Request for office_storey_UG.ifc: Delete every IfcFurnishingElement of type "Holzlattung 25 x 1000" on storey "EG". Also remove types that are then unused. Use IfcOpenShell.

First a look at what the model holds.

```python
import ifcopenshell
import ifcopenshell.util.element

model = ifcopenshell.open("office_storey_UG.ifc")
print(model.schema)
storey = next(s for s in model.by_type("IfcBuildingStorey") if s.Name == "EG")
furniture = [e for e in ifcopenshell.util.element.get_decomposition(storey) if e.is_a("IfcFurnishingElement")]
seen = {}
for e in furniture:
    element_type = ifcopenshell.util.element.get_type(e)
    name = element_type.Name if element_type not in (None, e) else None
    seen[name] = seen.get(name, 0) + 1
for name, count in sorted(seen.items(), key=str):
    print(count, "x", name)
```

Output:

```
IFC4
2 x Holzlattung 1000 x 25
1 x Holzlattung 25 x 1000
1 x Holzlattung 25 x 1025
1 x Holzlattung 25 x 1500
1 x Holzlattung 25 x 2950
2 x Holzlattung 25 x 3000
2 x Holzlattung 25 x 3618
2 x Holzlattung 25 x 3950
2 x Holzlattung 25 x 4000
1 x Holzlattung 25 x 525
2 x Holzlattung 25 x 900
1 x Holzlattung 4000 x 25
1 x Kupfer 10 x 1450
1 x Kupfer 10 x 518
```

```python
import ifcopenshell
import ifcopenshell.api.root
import ifcopenshell.util.element

model = ifcopenshell.open("office_storey_UG.ifc")

storey = next(s for s in model.by_type("IfcBuildingStorey") if s.Name == "EG")
furniture = [e for e in ifcopenshell.util.element.get_decomposition(storey) if e.is_a("IfcFurnishingElement")]
targets = [e for e in furniture if (t := ifcopenshell.util.element.get_type(e)) not in (None, e) and t.Name == "Holzlattung 25 x 1000"]
types = {ifcopenshell.util.element.get_type(e) for e in targets} - {None, *targets}

for e in targets:
    ifcopenshell.api.root.remove_product(model, product=e)
print(len(targets), "removed")

unused = [t for t in types if not ifcopenshell.util.element.get_types(t)]
for t in unused:
    ifcopenshell.api.root.remove_product(model, product=t)
print(len(unused), "unused types removed")

model.write("office_storey_UG_rev.ifc")
```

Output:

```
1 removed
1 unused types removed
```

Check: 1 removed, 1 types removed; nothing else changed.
